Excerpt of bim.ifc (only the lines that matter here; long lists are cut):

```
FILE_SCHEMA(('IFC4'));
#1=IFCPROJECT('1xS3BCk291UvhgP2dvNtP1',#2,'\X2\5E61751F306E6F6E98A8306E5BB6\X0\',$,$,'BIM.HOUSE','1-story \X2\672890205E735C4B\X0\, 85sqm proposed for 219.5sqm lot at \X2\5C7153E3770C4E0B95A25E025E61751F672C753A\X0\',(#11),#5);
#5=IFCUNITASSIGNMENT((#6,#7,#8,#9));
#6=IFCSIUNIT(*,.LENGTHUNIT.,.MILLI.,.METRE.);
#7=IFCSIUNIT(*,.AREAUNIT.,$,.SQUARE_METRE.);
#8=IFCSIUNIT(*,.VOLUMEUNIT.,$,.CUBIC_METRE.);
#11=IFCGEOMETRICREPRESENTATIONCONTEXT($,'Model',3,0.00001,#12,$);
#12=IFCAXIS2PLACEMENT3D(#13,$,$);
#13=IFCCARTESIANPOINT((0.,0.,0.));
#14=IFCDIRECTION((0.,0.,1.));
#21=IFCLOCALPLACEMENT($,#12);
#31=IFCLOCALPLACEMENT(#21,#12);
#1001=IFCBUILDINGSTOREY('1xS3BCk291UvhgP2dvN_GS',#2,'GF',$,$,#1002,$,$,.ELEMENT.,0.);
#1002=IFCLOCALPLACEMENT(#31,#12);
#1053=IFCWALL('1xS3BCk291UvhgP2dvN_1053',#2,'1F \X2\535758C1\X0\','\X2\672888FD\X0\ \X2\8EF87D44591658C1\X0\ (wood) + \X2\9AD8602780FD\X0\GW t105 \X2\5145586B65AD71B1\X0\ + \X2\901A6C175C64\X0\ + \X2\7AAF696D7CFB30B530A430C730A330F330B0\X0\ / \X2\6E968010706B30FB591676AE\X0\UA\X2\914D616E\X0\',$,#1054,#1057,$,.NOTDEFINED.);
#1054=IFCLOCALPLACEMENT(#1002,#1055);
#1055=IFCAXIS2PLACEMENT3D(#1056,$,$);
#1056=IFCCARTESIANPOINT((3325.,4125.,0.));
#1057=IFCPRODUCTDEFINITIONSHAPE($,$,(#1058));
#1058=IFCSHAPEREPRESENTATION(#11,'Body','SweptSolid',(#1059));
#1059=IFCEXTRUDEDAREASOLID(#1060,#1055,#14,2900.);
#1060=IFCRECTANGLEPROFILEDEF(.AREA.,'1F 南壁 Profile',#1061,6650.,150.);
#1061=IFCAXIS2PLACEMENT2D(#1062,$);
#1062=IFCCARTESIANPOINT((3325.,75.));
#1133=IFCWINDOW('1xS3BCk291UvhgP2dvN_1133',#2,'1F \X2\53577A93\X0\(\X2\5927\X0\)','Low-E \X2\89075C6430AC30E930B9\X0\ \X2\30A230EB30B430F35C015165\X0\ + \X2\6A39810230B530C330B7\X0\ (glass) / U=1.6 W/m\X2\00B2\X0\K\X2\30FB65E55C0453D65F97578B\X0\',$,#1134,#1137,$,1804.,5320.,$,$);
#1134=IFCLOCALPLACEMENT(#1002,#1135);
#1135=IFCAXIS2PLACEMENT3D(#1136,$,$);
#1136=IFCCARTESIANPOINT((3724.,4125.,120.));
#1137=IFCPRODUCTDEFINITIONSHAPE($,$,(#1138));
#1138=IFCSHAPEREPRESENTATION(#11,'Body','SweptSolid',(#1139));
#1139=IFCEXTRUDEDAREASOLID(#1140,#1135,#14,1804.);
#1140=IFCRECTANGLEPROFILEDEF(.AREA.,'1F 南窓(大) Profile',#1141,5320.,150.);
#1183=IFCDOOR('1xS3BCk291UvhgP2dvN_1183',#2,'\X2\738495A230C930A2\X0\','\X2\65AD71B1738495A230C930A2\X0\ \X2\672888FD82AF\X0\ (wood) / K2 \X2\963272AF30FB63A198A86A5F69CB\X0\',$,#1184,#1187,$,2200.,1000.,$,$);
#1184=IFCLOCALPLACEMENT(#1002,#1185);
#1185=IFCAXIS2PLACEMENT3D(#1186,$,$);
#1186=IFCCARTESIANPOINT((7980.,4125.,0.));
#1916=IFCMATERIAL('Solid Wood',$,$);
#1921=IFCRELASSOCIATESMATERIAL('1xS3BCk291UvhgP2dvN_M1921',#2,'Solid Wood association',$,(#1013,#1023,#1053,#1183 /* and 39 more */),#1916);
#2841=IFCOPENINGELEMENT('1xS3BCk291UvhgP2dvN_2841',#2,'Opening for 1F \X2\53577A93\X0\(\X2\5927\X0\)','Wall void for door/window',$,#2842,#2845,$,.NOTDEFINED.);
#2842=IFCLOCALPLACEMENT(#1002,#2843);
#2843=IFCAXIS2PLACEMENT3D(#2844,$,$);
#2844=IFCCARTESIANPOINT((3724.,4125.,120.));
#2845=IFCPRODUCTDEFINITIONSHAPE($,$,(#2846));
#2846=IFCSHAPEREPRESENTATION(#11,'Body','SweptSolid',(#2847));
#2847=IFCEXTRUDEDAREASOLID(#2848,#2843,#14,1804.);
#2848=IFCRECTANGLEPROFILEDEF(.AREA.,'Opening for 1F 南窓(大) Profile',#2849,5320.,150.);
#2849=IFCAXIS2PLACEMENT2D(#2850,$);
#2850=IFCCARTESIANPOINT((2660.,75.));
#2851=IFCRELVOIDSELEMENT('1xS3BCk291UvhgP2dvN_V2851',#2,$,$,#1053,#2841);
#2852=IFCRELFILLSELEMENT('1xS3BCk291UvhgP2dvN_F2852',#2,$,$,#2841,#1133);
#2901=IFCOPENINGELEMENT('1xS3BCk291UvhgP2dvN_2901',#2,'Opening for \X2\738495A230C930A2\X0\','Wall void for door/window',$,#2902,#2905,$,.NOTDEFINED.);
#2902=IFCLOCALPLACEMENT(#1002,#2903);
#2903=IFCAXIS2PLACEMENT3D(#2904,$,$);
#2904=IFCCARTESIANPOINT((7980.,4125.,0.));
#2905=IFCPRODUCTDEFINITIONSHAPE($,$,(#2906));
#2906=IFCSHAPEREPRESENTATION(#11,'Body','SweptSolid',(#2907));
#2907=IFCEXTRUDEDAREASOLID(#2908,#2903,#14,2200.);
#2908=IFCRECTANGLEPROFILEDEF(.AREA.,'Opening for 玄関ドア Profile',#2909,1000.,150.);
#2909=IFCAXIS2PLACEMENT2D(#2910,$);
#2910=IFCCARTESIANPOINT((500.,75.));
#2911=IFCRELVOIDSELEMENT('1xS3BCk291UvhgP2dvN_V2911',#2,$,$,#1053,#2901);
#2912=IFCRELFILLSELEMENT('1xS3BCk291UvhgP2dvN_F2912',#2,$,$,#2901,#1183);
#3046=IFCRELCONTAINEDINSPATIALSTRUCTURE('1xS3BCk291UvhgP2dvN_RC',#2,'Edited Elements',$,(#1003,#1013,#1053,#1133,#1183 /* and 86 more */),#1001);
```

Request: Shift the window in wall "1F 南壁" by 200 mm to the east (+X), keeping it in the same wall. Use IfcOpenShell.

```python
import ifcopenshell
import ifcopenshell.api.geometry
import ifcopenshell.util.placement
import ifcopenshell.util.unit

model = ifcopenshell.open("bim.ifc")
unit_scale = ifcopenshell.util.unit.calculate_unit_scale(model)

window = model.by_guid("1xS3BCk291UvhgP2dvN_1133")
opening = window.FillsVoids[0].RelatingOpeningElement
wall = opening.VoidsElements[0].RelatingBuildingElement

wall_matrix = ifcopenshell.util.placement.get_local_placement(wall.ObjectPlacement)
shift = wall_matrix[:3, 0] * 0.2 / unit_scale
before = ifcopenshell.util.placement.get_local_placement(window.ObjectPlacement)[:3, 3].copy()

# The window is not placed relative to its opening, so move both.
for product in (opening, window):
    matrix = ifcopenshell.util.placement.get_local_placement(product.ObjectPlacement)
    matrix[:3, 3] += shift
    ifcopenshell.api.geometry.edit_object_placement(model, product=product, matrix=matrix, is_si=False)

after = ifcopenshell.util.placement.get_local_placement(window.ObjectPlacement)[:3, 3]
print("window moved by", (after - before).round(3) + 0.0)

model.write("bim_updated.ifc")
```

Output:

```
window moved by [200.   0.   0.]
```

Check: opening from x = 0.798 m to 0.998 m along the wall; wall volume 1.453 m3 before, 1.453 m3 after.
